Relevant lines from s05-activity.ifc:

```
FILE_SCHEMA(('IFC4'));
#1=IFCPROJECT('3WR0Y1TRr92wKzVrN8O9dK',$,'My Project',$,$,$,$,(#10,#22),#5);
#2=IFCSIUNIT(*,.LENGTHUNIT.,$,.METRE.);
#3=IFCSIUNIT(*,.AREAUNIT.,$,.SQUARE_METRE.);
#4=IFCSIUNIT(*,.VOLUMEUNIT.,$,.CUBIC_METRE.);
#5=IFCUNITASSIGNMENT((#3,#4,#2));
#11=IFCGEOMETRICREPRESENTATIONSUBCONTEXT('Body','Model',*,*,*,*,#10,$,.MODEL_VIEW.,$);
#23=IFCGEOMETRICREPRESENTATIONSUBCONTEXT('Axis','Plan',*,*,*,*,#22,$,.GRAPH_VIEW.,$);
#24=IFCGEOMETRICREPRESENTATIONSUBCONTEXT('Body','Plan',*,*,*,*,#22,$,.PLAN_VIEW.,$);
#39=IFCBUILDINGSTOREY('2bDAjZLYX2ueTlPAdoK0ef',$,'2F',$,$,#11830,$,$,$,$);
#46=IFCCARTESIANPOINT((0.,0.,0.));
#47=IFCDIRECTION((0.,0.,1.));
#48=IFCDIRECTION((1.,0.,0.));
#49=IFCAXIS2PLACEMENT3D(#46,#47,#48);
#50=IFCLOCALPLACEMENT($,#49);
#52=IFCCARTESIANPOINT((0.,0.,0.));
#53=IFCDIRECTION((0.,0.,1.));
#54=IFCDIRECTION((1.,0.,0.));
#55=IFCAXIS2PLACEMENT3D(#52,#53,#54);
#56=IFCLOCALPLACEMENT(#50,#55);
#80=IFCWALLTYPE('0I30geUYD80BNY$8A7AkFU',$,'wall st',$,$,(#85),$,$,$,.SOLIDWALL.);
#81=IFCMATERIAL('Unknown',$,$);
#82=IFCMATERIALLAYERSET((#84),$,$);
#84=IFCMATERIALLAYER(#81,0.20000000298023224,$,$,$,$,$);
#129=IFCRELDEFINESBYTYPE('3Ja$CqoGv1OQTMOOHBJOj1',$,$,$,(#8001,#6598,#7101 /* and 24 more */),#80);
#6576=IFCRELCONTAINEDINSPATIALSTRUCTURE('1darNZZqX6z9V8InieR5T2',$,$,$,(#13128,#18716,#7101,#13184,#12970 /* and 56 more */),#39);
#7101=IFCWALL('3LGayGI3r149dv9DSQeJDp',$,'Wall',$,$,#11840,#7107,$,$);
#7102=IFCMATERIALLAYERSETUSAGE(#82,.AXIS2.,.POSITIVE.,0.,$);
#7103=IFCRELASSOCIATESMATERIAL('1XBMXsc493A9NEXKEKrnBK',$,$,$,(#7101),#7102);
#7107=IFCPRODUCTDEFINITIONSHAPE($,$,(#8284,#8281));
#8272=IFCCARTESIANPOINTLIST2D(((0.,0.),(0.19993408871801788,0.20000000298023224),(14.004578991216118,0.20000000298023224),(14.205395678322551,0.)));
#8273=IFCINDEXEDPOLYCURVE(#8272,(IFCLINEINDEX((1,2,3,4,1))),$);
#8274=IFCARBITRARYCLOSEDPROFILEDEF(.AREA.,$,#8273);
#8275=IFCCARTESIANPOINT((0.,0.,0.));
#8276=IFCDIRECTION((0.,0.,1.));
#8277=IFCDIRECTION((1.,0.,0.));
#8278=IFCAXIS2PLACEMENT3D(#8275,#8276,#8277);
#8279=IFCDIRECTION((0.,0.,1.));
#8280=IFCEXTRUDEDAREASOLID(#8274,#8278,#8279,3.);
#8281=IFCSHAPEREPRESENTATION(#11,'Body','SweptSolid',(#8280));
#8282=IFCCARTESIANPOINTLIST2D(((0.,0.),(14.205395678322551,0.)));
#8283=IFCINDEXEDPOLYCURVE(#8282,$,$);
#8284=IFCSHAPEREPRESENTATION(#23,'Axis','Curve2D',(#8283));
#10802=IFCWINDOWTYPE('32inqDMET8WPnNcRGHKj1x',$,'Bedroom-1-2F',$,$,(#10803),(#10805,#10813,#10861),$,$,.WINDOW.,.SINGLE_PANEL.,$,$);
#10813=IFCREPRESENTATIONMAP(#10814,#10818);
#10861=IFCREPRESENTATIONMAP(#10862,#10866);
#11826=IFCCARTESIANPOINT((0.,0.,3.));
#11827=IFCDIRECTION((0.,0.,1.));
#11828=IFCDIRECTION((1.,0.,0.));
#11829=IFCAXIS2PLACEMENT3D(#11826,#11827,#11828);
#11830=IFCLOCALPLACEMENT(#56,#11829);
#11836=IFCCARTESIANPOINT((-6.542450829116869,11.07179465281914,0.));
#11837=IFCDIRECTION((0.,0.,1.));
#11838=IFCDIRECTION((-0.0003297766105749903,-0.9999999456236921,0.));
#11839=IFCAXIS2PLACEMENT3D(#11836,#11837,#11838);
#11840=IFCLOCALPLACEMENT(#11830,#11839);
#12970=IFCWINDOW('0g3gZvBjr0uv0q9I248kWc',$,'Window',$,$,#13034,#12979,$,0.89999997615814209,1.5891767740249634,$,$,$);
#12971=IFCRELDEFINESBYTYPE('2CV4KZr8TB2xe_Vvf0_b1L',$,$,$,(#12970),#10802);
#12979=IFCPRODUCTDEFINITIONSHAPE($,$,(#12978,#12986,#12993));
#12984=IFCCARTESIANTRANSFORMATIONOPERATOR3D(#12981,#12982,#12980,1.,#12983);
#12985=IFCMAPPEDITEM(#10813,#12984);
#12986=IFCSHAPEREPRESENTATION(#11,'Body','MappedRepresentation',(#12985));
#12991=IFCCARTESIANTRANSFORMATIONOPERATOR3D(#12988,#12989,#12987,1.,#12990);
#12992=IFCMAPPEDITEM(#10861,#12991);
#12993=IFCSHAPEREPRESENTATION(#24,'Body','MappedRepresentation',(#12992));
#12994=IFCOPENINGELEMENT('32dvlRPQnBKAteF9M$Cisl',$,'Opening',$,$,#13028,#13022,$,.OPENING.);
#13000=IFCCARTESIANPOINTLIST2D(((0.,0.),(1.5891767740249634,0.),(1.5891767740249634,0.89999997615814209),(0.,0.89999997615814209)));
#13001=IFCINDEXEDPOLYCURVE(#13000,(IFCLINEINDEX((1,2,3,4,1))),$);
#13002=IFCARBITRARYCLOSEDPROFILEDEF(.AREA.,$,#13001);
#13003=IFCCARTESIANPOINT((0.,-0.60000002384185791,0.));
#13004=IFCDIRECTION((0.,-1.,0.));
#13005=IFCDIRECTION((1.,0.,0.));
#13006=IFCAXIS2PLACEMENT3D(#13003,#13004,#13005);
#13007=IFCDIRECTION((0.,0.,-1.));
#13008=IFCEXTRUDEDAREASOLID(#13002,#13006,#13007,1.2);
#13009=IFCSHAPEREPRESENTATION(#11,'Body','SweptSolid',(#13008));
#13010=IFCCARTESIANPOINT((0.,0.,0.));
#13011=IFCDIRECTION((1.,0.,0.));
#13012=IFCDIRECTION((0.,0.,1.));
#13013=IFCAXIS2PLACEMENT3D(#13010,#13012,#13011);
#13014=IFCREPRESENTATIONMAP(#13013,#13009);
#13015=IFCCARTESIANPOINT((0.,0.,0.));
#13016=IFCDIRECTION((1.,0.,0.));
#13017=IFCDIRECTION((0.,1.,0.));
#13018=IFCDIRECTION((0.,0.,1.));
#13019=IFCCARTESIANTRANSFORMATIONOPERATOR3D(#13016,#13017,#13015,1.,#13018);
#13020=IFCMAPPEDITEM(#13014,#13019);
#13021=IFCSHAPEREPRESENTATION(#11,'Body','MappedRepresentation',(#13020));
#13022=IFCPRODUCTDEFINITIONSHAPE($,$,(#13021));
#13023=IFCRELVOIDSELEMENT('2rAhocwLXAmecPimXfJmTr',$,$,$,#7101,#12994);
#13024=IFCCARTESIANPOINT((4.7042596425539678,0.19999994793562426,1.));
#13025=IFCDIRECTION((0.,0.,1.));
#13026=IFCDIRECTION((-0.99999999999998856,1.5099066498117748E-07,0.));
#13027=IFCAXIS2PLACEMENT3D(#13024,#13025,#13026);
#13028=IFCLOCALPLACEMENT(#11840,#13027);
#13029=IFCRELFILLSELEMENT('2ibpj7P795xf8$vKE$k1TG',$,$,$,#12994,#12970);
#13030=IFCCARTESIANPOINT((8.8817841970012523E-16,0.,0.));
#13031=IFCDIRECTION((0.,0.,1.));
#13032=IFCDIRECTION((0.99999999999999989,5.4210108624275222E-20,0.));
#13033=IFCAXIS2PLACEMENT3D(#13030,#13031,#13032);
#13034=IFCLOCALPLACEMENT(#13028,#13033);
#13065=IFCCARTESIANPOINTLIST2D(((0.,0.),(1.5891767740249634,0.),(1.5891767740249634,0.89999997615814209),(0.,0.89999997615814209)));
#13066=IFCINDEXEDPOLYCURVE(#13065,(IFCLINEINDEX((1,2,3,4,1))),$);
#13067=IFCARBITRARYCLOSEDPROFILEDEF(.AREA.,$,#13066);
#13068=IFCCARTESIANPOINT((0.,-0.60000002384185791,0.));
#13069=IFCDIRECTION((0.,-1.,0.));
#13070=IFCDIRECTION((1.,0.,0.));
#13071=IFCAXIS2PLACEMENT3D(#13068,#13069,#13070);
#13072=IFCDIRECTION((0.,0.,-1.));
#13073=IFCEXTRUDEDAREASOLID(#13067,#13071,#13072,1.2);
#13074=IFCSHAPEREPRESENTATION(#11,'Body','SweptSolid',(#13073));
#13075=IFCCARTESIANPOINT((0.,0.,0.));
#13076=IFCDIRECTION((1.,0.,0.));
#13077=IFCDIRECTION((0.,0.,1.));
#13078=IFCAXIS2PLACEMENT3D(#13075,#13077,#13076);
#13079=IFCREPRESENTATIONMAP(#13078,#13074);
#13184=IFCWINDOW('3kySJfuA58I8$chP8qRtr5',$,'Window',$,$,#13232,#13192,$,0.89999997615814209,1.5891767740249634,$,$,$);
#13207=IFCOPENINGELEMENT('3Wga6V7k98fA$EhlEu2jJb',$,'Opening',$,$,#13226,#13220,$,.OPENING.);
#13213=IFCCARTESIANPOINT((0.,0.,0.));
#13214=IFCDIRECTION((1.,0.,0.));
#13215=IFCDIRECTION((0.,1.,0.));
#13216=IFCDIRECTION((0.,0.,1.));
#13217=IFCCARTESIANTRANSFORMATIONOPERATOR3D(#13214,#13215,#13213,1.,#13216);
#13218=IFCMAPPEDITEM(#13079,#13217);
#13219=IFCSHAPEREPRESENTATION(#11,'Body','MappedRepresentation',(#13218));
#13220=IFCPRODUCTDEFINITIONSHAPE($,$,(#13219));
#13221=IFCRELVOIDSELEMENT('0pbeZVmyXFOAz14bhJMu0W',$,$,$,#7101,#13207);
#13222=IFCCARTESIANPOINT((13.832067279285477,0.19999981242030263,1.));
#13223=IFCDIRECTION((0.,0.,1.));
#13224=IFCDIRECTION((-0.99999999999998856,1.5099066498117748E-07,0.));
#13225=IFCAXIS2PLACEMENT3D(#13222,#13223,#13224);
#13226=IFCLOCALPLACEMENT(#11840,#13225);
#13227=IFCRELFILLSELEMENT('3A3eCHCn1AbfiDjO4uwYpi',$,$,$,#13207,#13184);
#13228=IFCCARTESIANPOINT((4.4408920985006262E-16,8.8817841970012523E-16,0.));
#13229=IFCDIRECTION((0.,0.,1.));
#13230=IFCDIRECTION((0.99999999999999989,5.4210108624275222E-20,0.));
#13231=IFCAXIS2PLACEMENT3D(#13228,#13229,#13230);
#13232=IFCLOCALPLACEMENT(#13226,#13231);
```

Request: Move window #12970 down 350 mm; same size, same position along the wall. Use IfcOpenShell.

```python
import numpy as np
import ifcopenshell
import ifcopenshell.api.geometry
import ifcopenshell.util.placement
import ifcopenshell.util.unit

model = ifcopenshell.open("s05-activity.ifc")
unit_scale = ifcopenshell.util.unit.calculate_unit_scale(model)

window = model.by_guid("0g3gZvBjr0uv0q9I248kWc")
opening = window.FillsVoids[0].RelatingOpeningElement
dz = -0.35 / unit_scale

shift = np.array([0.0, 0.0, dz])
# The window is placed relative to its opening, so it follows when the opening moves.
matrix = ifcopenshell.util.placement.get_local_placement(opening.ObjectPlacement)
matrix[:3, 3] += shift
ifcopenshell.api.geometry.edit_object_placement(
    model, product=opening, matrix=matrix, is_si=False, should_transform_children=True
)

print(f"moved by {dz * unit_scale:+.3f} m")

model.write("s05-activity_v2.ifc")
```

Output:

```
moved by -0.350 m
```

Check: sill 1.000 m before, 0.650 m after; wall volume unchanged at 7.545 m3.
